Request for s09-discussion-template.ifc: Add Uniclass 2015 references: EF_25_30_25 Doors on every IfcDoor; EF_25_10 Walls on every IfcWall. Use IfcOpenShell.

First a look at what the model holds.

```python
import ifcopenshell

model = ifcopenshell.open("s09-discussion-template.ifc")
print(model.schema)
print("classifications:", [c.Name for c in model.by_type("IfcClassification")])
for ifc_class in ("IfcDoor", "IfcRoof", "IfcStair", "IfcWall", "IfcWindow"):
    print(ifc_class, len(model.by_type(ifc_class)))
```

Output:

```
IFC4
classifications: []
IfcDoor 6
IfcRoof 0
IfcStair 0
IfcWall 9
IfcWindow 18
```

```python
import ifcopenshell
import ifcopenshell.api.classification

model = ifcopenshell.open("s09-discussion-template.ifc")

system = ifcopenshell.api.classification.add_classification(model, classification="Uniclass 2015")

codes = {
    "IfcDoor": ("EF_25_30_25", "Doors"),
    "IfcWall": ("EF_25_10", "Walls"),
}
for ifc_class, (code, name) in codes.items():
    products = model.by_type(ifc_class)
    ifcopenshell.api.classification.add_reference(
        model, products=products, classification=system, identification=code, name=name
    )
    print(code, len(products))

model.write("s09-discussion-template_updated.ifc")
```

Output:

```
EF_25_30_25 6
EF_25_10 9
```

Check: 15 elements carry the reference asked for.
